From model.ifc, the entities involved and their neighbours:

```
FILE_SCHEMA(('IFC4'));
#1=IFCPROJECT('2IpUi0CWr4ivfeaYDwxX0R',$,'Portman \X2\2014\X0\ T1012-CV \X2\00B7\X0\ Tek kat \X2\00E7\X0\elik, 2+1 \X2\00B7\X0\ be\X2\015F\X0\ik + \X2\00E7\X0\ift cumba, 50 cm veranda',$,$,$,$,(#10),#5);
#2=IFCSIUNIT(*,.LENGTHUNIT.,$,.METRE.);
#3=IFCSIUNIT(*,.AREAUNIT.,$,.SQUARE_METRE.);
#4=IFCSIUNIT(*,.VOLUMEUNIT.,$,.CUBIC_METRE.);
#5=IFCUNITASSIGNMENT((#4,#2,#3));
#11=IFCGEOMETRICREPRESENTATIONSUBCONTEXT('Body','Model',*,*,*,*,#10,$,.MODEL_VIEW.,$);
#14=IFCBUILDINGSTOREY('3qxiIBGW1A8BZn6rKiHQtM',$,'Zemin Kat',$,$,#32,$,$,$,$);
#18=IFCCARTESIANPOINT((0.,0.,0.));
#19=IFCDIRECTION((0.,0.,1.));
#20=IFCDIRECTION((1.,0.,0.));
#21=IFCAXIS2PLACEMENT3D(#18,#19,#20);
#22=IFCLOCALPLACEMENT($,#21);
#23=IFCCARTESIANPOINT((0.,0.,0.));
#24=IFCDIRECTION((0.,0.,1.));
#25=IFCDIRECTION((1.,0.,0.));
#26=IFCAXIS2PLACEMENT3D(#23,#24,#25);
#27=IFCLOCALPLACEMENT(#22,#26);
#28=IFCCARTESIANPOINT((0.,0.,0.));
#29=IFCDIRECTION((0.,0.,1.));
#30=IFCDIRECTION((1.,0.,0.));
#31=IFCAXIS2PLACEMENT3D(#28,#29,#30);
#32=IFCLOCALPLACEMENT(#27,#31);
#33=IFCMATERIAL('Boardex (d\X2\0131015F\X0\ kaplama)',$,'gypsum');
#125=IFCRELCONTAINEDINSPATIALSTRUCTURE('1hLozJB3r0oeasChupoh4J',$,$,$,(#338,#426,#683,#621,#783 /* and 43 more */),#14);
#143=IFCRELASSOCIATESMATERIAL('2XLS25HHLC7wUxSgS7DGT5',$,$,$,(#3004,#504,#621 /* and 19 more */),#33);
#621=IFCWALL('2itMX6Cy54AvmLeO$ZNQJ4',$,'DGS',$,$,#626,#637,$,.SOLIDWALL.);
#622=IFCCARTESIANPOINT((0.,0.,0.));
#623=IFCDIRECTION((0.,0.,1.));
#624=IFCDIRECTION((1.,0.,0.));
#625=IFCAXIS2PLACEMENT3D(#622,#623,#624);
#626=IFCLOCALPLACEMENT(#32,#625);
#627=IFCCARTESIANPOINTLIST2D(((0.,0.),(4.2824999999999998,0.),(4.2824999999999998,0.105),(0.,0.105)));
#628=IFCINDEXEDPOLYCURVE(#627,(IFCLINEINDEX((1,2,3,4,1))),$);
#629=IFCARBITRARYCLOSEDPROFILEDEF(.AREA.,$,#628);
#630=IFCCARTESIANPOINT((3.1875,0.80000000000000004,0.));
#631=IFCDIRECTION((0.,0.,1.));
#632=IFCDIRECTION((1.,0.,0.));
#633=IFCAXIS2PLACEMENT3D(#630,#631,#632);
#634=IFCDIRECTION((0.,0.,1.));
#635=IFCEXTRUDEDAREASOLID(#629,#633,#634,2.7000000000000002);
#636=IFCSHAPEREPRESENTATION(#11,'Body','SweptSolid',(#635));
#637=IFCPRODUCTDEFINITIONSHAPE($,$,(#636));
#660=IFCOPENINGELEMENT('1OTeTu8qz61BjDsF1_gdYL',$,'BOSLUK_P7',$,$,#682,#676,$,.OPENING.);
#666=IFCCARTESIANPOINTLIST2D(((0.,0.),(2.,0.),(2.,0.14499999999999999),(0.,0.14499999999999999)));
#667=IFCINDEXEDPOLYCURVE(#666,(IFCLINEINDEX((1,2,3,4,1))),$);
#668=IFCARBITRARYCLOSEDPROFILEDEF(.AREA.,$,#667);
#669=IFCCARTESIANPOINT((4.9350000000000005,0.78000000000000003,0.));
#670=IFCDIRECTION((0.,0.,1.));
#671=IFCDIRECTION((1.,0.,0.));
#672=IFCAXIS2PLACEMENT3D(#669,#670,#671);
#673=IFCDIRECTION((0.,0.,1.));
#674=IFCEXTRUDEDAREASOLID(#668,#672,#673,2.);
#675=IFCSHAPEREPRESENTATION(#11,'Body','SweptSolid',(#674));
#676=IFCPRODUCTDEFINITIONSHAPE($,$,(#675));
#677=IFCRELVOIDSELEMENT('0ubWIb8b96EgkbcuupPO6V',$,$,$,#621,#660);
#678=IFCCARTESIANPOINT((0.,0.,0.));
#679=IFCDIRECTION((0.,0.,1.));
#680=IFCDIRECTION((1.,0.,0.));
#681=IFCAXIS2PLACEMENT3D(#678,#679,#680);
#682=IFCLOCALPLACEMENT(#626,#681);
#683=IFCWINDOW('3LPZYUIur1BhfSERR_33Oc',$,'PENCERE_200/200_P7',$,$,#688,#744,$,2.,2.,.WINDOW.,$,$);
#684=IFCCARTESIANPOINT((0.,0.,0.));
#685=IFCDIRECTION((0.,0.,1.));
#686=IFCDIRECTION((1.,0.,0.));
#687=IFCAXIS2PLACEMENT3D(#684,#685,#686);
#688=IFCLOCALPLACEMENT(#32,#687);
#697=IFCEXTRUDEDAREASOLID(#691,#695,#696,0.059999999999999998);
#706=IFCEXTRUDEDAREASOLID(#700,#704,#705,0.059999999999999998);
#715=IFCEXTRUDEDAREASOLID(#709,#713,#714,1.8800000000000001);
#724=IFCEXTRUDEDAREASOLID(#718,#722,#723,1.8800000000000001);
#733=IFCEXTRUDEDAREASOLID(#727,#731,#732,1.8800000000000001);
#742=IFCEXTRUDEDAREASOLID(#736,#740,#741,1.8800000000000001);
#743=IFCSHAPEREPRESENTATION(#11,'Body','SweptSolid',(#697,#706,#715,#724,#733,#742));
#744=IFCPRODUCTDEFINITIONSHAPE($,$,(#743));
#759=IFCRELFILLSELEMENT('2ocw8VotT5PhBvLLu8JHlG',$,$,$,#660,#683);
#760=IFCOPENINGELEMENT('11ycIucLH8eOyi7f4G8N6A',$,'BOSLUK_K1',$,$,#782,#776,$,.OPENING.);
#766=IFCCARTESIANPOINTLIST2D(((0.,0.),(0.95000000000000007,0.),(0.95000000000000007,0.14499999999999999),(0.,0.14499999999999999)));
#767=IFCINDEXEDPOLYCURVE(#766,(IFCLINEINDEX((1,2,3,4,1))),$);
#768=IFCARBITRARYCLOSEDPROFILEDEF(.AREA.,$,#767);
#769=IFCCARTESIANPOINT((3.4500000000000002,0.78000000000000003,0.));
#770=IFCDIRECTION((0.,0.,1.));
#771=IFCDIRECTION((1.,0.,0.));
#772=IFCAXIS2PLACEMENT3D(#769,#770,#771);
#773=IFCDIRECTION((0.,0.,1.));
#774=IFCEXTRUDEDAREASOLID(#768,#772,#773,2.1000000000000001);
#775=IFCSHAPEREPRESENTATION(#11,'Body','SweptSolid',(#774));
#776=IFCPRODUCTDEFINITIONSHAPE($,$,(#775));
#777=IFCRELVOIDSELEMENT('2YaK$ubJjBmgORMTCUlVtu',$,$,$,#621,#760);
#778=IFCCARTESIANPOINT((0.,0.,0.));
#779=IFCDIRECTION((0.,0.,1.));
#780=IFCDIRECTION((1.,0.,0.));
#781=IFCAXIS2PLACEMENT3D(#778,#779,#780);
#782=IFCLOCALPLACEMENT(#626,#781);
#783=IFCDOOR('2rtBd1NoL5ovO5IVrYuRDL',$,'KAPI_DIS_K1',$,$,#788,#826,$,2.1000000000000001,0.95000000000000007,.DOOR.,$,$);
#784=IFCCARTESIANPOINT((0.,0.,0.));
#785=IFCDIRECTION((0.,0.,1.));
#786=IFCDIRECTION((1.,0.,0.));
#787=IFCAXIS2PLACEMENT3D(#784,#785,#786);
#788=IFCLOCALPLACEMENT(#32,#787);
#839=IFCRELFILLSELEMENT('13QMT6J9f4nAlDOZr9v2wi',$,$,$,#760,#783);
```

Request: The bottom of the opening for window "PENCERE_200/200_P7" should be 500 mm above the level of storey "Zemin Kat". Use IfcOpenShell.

```python
import numpy as np
import ifcopenshell
import ifcopenshell.api.geometry
import ifcopenshell.geom
import ifcopenshell.util.element
import ifcopenshell.util.placement
import ifcopenshell.util.shape
import ifcopenshell.util.unit

model = ifcopenshell.open("model.ifc")
unit_scale = ifcopenshell.util.unit.calculate_unit_scale(model)

window = model.by_guid("3LPZYUIur1BhfSERR_33Oc")
opening = window.FillsVoids[0].RelatingOpeningElement
storey = ifcopenshell.util.element.get_container(window, ifc_class="IfcBuildingStorey")
level = ifcopenshell.util.placement.get_local_placement(storey.ObjectPlacement)[2, 3]

# The opening's origin need not be at the sill, so measure its lowest point.
shape = ifcopenshell.geom.create_shape(ifcopenshell.geom.settings(), opening)
bottom = ifcopenshell.util.shape.get_shape_bottom_elevation(shape, shape.geometry) / unit_scale
dz = level + 0.5 - bottom

shift = np.array([0.0, 0.0, dz])
# The window is not placed relative to its opening, so move both.
for product in (opening, window):
    matrix = ifcopenshell.util.placement.get_local_placement(product.ObjectPlacement)
    matrix[:3, 3] += shift
    ifcopenshell.api.geometry.edit_object_placement(model, product=product, matrix=matrix, is_si=False)

print(f"moved by {dz * unit_scale:+.3f} m")

model.write("model_v2.ifc")
```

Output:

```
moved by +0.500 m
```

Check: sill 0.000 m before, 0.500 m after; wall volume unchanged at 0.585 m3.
